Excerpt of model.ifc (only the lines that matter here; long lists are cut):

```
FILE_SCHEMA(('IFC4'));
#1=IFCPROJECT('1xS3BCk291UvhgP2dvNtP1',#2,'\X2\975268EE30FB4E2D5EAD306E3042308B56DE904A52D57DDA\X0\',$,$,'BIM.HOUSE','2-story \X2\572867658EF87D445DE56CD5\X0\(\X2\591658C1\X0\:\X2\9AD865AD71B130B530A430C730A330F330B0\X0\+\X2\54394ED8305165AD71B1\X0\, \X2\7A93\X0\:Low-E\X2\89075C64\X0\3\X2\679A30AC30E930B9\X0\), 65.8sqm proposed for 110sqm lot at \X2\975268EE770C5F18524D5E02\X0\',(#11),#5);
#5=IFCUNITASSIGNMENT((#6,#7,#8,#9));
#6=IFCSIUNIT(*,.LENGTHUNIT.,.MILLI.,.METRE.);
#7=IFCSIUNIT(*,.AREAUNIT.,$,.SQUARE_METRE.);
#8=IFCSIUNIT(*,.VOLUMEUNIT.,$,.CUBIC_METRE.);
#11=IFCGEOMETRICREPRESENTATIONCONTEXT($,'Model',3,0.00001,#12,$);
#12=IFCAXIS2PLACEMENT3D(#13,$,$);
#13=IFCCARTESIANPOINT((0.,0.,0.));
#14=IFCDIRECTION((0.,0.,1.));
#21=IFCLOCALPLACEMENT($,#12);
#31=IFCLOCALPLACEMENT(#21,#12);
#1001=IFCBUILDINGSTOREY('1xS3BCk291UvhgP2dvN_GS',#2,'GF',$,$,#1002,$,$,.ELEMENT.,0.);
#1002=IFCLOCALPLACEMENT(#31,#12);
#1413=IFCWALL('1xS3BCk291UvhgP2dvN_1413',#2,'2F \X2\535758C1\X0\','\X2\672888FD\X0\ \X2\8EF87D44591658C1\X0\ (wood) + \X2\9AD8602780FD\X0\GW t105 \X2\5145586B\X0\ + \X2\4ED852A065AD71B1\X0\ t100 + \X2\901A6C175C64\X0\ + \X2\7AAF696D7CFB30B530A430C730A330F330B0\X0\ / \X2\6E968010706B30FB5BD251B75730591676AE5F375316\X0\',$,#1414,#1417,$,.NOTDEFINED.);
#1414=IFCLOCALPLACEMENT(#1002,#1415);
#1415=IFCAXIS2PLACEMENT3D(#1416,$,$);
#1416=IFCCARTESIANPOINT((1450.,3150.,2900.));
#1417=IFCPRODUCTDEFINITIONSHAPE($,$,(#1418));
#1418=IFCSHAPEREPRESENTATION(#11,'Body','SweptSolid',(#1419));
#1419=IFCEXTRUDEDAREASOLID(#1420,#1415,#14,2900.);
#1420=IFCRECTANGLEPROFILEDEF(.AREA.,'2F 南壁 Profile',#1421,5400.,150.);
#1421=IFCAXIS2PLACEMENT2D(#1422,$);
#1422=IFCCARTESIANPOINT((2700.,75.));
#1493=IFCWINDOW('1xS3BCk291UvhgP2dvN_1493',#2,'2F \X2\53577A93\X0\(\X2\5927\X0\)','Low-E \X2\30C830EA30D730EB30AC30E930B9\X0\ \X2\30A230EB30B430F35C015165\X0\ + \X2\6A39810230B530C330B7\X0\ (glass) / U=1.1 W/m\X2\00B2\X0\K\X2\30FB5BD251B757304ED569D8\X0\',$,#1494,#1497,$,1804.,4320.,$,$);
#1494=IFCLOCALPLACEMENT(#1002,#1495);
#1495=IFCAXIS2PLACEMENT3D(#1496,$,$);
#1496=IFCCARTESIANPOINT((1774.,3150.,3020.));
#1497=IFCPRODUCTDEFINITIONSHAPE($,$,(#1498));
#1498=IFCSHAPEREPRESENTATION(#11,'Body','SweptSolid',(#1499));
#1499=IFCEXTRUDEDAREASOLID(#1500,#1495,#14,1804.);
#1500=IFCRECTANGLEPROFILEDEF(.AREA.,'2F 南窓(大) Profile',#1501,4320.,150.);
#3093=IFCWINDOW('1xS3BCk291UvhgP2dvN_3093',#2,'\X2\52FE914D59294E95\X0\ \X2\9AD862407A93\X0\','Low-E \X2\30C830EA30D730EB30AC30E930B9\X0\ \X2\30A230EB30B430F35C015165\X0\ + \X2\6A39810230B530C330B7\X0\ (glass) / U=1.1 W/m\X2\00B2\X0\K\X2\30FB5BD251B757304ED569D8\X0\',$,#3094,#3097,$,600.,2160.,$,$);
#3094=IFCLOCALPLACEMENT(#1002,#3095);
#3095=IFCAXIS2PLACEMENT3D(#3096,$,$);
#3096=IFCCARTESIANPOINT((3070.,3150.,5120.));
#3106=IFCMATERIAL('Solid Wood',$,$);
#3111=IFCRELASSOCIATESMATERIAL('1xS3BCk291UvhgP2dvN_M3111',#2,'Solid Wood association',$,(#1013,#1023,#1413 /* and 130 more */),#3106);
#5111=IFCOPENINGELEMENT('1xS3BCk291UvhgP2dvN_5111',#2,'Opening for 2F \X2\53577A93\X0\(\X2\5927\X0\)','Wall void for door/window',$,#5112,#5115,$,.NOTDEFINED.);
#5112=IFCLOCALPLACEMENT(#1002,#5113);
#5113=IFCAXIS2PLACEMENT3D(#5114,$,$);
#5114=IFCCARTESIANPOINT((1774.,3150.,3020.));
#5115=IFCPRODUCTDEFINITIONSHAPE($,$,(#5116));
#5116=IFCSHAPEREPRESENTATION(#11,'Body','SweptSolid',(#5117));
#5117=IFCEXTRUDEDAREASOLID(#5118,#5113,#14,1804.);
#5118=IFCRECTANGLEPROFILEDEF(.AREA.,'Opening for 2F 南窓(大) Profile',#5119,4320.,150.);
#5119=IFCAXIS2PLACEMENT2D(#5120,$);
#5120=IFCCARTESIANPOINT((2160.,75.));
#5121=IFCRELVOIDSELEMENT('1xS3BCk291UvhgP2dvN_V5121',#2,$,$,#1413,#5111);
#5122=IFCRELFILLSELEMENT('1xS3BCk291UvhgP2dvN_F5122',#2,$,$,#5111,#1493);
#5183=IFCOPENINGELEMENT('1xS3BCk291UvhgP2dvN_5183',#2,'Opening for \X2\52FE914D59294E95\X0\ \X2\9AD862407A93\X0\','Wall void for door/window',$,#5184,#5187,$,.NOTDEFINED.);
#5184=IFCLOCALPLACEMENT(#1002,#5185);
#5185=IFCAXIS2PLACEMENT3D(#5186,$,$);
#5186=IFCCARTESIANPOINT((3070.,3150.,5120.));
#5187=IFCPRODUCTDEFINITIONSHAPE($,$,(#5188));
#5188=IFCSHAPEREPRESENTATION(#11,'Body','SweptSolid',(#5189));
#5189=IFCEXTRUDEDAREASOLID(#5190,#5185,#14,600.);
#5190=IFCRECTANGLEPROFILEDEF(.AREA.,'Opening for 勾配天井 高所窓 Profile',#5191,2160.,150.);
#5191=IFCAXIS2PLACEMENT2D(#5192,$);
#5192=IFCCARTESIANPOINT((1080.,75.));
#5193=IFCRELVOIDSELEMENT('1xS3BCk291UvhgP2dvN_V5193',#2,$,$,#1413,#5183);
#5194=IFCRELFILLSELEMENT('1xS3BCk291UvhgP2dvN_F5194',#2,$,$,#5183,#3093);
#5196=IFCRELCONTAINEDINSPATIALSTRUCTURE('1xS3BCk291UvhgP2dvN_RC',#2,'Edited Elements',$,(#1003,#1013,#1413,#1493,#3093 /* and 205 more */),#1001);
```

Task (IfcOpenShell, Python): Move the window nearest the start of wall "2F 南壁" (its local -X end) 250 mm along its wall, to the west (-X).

```python
import ifcopenshell
import ifcopenshell.api.geometry
import ifcopenshell.util.placement

model = ifcopenshell.open("model.ifc")

window = model.by_guid("1xS3BCk291UvhgP2dvN_1493")
opening = window.FillsVoids[0].RelatingOpeningElement
wall = opening.VoidsElements[0].RelatingBuildingElement

wall_matrix = ifcopenshell.util.placement.get_local_placement(wall.ObjectPlacement)
shift = wall_matrix[:3, 0] * -250.0
before = ifcopenshell.util.placement.get_local_placement(window.ObjectPlacement)[:3, 3].copy()

# The window is not placed relative to its opening, so move both.
for product in (opening, window):
    matrix = ifcopenshell.util.placement.get_local_placement(product.ObjectPlacement)
    matrix[:3, 3] += shift
    ifcopenshell.api.geometry.edit_object_placement(model, product=product, matrix=matrix, is_si=False)

after = ifcopenshell.util.placement.get_local_placement(window.ObjectPlacement)[:3, 3]
print("window moved by", (after - before).round(3) + 0.0)

model.write("model_updated.ifc")
```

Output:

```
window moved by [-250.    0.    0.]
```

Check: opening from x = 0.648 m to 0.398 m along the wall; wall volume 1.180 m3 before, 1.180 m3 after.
